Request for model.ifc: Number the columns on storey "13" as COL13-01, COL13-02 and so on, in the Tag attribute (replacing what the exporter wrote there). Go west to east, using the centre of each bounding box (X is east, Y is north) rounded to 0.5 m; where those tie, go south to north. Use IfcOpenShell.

First a look at what the model holds.

```python
import ifcopenshell
import ifcopenshell.util.element
import ifcopenshell.util.placement

model = ifcopenshell.open("model.ifc")
print(model.schema)
storey = next(s for s in model.by_type("IfcBuildingStorey") if s.Name == "13")
columns = [e for e in ifcopenshell.util.element.get_decomposition(storey) if e.is_a("IfcColumn")]
for e in sorted(columns, key=lambda e: e.id()):
    origin = ifcopenshell.util.placement.get_local_placement(e.ObjectPlacement)[:3, 3]
    print(e.id(), e.Tag, e.Name, origin.round(2) + 0.0, sep=" | ")
```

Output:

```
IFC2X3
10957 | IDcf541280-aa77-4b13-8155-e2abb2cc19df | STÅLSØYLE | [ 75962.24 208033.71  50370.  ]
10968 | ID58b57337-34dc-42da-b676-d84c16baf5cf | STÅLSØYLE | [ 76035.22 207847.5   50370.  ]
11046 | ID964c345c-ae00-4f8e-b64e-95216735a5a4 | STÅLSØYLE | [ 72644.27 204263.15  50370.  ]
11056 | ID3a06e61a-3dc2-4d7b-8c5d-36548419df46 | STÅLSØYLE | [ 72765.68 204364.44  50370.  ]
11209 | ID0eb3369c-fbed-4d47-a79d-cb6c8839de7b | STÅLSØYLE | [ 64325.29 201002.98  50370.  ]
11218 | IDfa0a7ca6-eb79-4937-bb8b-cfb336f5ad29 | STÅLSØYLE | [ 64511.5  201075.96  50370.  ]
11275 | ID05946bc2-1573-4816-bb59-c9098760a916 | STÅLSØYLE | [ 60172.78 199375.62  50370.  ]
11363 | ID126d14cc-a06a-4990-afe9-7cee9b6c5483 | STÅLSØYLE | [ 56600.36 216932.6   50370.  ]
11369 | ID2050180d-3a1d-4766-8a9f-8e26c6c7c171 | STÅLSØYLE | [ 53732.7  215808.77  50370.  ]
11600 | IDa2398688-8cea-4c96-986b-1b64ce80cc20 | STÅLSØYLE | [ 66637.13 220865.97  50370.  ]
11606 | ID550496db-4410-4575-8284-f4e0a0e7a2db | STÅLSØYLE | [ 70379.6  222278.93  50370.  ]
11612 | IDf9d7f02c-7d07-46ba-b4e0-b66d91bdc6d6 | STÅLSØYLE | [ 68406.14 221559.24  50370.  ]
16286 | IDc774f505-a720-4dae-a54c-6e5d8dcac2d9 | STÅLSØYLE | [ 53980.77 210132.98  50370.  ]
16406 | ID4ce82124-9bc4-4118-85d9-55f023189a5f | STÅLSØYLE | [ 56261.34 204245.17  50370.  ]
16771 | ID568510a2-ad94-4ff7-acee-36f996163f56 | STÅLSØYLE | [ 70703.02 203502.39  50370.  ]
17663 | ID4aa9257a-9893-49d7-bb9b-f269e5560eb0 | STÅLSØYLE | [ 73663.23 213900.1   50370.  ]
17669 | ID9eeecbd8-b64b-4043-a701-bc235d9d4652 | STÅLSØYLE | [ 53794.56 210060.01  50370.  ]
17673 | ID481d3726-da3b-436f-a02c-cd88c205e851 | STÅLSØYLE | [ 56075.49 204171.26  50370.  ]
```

```python
import ifcopenshell
import ifcopenshell.geom
import ifcopenshell.util.element
import ifcopenshell.util.shape

model = ifcopenshell.open("model.ifc")
settings = ifcopenshell.geom.settings()
settings.set("use-world-coords", True)


def centre(element):
    shape = ifcopenshell.geom.create_shape(settings, element)
    return ifcopenshell.util.shape.get_bbox_centroid(shape.geometry)


storey = next(s for s in model.by_type("IfcBuildingStorey") if s.Name == "13")
columns = [e for e in ifcopenshell.util.element.get_decomposition(storey) if e.is_a("IfcColumn")]

# Insertion points can sit at a corner or the storey origin, so sort by the geometry (in metres).
centres = {e: centre(e) for e in columns}
columns.sort(key=lambda e: (round(centres[e][0] / 0.5), centres[e][1]))

for i, e in enumerate(columns, start=1):
    number = f"COL13-{i:02d}"
    e.Tag = number
    print(e.id(), number)

model.write("model_rev.ifc")
```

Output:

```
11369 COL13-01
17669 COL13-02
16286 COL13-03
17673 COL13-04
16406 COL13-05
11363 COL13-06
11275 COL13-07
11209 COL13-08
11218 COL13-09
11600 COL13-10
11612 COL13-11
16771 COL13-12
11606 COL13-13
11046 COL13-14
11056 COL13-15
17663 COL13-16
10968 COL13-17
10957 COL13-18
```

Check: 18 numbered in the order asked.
